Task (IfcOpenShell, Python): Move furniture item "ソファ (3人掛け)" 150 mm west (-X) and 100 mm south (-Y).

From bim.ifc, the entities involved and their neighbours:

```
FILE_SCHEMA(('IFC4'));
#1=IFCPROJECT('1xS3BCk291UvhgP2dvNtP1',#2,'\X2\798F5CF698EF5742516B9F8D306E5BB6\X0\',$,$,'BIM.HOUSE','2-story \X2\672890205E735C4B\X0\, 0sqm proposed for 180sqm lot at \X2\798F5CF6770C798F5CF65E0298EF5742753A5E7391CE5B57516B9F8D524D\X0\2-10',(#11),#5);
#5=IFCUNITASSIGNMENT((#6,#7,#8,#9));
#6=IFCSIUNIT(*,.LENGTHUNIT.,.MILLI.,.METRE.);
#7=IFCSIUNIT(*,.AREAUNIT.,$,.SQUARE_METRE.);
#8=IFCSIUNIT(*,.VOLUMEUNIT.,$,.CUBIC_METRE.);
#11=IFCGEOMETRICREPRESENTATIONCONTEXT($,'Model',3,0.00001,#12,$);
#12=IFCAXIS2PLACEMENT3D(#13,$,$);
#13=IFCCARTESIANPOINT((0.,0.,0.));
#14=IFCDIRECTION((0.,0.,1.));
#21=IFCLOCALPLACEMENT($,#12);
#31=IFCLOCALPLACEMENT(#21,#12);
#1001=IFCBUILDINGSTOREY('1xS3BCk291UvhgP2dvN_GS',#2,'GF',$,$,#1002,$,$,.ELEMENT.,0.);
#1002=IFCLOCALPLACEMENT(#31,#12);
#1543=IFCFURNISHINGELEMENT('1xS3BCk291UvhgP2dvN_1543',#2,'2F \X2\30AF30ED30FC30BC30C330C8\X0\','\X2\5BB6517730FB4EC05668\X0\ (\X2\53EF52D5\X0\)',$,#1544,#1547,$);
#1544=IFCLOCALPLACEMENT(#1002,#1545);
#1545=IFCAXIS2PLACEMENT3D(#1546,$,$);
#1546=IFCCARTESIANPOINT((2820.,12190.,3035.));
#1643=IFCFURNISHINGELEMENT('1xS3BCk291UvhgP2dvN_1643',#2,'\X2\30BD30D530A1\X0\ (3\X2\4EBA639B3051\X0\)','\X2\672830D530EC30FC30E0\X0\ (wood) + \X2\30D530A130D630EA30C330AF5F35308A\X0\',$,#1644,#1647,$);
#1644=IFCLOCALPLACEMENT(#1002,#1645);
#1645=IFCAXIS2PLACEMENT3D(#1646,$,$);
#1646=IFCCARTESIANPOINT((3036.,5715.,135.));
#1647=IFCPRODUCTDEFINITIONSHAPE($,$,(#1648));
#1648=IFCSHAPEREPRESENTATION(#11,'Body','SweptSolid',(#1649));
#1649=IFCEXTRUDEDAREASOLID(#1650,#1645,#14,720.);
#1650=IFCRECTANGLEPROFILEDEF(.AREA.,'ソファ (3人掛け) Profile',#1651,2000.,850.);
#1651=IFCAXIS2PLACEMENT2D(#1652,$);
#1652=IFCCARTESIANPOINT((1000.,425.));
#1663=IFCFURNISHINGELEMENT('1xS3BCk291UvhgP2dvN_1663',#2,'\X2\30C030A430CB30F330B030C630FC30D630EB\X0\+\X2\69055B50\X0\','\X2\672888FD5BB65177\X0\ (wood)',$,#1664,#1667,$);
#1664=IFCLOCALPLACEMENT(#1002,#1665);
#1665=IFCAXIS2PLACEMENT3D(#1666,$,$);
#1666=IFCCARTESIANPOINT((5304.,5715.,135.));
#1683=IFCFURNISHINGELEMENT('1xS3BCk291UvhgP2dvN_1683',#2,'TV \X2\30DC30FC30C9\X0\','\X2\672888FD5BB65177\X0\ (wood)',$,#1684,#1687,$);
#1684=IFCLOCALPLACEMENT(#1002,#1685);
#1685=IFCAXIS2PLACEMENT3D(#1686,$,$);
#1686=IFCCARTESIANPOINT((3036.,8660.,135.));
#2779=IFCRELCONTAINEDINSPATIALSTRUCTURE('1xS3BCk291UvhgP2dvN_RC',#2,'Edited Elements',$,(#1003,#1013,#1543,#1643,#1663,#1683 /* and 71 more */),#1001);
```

```python
import ifcopenshell
import ifcopenshell.api.geometry
import ifcopenshell.util.placement
import ifcopenshell.util.unit

model = ifcopenshell.open("bim.ifc")
unit_scale = ifcopenshell.util.unit.calculate_unit_scale(model)

item = model.by_guid("1xS3BCk291UvhgP2dvN_1643")
matrix = ifcopenshell.util.placement.get_local_placement(item.ObjectPlacement)
matrix[0, 3] -= 0.15 / unit_scale
matrix[1, 3] -= 0.1 / unit_scale
ifcopenshell.api.geometry.edit_object_placement(model, product=item, matrix=matrix, is_si=False)

print(ifcopenshell.util.placement.get_local_placement(item.ObjectPlacement).round(3) + 0.0)

model.write("bim_edited.ifc")
```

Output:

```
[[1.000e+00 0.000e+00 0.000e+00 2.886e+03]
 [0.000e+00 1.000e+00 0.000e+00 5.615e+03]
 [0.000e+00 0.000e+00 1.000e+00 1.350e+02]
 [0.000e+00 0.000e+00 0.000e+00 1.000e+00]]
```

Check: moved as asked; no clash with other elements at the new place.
